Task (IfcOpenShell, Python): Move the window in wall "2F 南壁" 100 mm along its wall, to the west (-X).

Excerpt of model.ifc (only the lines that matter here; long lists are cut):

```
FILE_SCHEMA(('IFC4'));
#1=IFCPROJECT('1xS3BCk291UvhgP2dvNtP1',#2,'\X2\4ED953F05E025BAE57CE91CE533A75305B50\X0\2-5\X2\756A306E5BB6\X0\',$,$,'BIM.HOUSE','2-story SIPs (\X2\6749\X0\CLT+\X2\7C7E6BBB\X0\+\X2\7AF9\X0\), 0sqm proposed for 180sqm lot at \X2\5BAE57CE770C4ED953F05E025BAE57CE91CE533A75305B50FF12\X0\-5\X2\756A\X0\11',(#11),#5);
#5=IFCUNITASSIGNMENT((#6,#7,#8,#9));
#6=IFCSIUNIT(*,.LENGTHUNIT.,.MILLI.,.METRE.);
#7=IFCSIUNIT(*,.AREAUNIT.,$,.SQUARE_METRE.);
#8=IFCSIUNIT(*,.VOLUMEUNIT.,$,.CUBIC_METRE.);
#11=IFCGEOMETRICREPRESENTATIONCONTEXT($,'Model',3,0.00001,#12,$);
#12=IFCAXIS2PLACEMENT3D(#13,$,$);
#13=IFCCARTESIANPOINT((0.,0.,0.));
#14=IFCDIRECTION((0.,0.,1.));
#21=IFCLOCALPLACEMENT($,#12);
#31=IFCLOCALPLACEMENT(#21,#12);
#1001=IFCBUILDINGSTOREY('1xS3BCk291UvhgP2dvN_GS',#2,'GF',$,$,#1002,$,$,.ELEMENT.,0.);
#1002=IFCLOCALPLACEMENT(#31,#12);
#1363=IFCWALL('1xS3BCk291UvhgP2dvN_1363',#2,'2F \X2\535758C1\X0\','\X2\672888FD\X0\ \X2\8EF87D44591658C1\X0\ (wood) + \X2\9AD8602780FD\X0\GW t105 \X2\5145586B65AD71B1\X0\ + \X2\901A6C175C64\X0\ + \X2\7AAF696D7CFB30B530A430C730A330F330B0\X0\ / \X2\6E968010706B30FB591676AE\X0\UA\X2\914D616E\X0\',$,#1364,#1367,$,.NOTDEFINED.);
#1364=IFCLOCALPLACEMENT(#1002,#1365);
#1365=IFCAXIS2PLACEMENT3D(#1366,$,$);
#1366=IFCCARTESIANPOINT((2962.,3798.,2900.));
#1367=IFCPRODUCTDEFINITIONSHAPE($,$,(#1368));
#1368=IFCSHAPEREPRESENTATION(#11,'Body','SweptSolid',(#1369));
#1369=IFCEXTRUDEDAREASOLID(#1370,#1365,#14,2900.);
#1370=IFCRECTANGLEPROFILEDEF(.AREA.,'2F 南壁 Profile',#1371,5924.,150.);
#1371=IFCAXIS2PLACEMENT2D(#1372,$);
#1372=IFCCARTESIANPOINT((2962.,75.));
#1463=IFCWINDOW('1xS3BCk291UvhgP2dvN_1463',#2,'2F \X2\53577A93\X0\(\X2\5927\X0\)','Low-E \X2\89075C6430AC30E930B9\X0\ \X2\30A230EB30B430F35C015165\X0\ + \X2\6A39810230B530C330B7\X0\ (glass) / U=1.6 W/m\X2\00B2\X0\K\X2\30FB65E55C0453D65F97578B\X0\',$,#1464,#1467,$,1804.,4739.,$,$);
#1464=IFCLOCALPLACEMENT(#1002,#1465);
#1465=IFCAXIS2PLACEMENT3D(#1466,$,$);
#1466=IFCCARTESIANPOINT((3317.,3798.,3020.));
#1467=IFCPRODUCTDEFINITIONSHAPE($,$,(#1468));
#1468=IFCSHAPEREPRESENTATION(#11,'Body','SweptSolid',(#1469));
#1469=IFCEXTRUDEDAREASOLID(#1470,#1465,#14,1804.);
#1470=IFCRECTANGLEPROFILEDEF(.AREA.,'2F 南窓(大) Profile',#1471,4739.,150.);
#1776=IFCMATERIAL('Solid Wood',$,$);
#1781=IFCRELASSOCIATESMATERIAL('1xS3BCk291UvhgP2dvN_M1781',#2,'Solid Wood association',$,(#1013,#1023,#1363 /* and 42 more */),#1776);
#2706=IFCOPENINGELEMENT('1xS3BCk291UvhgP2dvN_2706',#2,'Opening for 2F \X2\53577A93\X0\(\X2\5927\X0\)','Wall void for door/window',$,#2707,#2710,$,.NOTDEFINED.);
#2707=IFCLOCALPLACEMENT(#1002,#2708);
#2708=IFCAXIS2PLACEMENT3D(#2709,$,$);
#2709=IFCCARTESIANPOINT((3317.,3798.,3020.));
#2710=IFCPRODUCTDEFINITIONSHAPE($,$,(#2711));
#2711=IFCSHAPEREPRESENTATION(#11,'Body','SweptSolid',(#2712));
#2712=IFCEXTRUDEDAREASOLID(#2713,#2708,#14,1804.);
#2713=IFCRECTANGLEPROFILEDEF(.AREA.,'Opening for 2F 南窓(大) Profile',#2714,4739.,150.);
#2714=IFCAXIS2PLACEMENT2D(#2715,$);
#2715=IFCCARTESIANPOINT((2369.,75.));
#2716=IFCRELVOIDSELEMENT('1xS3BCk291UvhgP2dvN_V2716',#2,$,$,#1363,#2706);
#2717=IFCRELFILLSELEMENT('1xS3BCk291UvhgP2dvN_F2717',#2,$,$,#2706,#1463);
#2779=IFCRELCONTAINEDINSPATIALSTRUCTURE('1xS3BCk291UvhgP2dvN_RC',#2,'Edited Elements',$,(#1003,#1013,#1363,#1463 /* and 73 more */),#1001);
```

```python
import ifcopenshell
import ifcopenshell.api.geometry
import ifcopenshell.util.placement
import ifcopenshell.util.unit

model = ifcopenshell.open("model.ifc")
unit_scale = ifcopenshell.util.unit.calculate_unit_scale(model)

window = model.by_guid("1xS3BCk291UvhgP2dvN_1463")
opening = window.FillsVoids[0].RelatingOpeningElement
wall = opening.VoidsElements[0].RelatingBuildingElement

wall_matrix = ifcopenshell.util.placement.get_local_placement(wall.ObjectPlacement)
shift = wall_matrix[:3, 0] * -0.1 / unit_scale
before = ifcopenshell.util.placement.get_local_placement(window.ObjectPlacement)[:3, 3].copy()

# The window is not placed relative to its opening, so move both.
for product in (opening, window):
    matrix = ifcopenshell.util.placement.get_local_placement(product.ObjectPlacement)
    matrix[:3, 3] += shift
    ifcopenshell.api.geometry.edit_object_placement(model, product=product, matrix=matrix, is_si=False)

after = ifcopenshell.util.placement.get_local_placement(window.ObjectPlacement)[:3, 3]
print("window moved by", (after - before).round(3) + 0.0)

model.write("model_updated.ifc")
```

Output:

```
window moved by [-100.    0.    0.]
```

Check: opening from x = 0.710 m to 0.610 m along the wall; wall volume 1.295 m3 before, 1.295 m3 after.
